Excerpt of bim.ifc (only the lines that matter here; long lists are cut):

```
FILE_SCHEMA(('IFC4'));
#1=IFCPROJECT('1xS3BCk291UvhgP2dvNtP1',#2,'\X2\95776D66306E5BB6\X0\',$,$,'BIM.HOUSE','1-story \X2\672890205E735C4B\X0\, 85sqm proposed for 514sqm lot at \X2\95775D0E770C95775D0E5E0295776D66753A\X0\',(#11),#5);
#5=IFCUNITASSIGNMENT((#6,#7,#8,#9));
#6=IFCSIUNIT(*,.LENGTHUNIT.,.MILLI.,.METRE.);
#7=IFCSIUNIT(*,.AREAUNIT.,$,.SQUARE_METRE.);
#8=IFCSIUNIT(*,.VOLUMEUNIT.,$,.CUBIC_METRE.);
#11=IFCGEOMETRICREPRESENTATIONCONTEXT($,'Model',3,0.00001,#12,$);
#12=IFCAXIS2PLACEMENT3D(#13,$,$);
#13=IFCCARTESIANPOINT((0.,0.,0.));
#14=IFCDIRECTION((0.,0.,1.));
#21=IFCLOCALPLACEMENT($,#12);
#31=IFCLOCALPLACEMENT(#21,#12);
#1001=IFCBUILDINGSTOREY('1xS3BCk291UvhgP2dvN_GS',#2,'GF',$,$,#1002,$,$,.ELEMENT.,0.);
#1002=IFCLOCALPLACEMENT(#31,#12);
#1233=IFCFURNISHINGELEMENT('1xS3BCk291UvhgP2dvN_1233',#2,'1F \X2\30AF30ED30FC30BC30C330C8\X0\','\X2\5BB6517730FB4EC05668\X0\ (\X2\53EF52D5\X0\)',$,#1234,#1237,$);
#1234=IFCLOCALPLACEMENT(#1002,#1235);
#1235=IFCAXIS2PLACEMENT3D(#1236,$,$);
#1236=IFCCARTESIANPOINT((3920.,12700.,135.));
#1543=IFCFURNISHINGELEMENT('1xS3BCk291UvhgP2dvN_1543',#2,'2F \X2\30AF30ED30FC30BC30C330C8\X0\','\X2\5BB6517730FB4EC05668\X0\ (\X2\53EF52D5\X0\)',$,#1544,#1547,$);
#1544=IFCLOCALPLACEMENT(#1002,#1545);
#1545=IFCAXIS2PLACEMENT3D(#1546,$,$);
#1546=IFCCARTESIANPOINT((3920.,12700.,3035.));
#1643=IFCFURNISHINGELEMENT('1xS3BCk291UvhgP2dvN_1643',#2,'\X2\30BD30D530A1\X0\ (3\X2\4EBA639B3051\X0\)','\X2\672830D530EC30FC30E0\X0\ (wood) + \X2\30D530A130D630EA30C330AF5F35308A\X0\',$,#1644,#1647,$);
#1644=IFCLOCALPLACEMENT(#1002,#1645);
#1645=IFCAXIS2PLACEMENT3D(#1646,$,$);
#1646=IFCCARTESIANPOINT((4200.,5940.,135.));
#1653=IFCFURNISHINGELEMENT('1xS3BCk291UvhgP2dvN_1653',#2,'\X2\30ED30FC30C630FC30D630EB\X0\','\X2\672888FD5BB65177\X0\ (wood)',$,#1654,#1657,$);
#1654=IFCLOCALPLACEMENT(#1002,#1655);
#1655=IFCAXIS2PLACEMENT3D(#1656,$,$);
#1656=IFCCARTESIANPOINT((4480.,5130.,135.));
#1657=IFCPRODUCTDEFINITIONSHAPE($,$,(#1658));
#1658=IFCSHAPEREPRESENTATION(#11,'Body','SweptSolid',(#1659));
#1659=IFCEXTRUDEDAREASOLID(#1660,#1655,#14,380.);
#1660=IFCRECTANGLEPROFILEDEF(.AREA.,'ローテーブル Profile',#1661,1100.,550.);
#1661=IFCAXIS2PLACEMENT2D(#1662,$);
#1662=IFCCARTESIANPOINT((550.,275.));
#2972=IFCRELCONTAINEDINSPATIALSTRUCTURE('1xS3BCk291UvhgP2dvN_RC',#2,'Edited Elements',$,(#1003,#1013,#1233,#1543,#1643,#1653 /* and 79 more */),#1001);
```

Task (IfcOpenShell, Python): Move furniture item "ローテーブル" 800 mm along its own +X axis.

```python
import ifcopenshell
import ifcopenshell.api.geometry
import ifcopenshell.util.placement

model = ifcopenshell.open("bim.ifc")

item = model.by_guid("1xS3BCk291UvhgP2dvN_1653")
matrix = ifcopenshell.util.placement.get_local_placement(item.ObjectPlacement)
matrix[:3, 3] += matrix[:3, 0] * 800.0
ifcopenshell.api.geometry.edit_object_placement(model, product=item, matrix=matrix, is_si=False)

print(ifcopenshell.util.placement.get_local_placement(item.ObjectPlacement).round(3) + 0.0)

model.write("bim_v2.ifc")
```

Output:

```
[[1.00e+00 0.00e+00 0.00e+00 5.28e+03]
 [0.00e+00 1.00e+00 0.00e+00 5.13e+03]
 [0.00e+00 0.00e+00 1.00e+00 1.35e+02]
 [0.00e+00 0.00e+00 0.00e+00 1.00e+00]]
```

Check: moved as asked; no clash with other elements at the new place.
